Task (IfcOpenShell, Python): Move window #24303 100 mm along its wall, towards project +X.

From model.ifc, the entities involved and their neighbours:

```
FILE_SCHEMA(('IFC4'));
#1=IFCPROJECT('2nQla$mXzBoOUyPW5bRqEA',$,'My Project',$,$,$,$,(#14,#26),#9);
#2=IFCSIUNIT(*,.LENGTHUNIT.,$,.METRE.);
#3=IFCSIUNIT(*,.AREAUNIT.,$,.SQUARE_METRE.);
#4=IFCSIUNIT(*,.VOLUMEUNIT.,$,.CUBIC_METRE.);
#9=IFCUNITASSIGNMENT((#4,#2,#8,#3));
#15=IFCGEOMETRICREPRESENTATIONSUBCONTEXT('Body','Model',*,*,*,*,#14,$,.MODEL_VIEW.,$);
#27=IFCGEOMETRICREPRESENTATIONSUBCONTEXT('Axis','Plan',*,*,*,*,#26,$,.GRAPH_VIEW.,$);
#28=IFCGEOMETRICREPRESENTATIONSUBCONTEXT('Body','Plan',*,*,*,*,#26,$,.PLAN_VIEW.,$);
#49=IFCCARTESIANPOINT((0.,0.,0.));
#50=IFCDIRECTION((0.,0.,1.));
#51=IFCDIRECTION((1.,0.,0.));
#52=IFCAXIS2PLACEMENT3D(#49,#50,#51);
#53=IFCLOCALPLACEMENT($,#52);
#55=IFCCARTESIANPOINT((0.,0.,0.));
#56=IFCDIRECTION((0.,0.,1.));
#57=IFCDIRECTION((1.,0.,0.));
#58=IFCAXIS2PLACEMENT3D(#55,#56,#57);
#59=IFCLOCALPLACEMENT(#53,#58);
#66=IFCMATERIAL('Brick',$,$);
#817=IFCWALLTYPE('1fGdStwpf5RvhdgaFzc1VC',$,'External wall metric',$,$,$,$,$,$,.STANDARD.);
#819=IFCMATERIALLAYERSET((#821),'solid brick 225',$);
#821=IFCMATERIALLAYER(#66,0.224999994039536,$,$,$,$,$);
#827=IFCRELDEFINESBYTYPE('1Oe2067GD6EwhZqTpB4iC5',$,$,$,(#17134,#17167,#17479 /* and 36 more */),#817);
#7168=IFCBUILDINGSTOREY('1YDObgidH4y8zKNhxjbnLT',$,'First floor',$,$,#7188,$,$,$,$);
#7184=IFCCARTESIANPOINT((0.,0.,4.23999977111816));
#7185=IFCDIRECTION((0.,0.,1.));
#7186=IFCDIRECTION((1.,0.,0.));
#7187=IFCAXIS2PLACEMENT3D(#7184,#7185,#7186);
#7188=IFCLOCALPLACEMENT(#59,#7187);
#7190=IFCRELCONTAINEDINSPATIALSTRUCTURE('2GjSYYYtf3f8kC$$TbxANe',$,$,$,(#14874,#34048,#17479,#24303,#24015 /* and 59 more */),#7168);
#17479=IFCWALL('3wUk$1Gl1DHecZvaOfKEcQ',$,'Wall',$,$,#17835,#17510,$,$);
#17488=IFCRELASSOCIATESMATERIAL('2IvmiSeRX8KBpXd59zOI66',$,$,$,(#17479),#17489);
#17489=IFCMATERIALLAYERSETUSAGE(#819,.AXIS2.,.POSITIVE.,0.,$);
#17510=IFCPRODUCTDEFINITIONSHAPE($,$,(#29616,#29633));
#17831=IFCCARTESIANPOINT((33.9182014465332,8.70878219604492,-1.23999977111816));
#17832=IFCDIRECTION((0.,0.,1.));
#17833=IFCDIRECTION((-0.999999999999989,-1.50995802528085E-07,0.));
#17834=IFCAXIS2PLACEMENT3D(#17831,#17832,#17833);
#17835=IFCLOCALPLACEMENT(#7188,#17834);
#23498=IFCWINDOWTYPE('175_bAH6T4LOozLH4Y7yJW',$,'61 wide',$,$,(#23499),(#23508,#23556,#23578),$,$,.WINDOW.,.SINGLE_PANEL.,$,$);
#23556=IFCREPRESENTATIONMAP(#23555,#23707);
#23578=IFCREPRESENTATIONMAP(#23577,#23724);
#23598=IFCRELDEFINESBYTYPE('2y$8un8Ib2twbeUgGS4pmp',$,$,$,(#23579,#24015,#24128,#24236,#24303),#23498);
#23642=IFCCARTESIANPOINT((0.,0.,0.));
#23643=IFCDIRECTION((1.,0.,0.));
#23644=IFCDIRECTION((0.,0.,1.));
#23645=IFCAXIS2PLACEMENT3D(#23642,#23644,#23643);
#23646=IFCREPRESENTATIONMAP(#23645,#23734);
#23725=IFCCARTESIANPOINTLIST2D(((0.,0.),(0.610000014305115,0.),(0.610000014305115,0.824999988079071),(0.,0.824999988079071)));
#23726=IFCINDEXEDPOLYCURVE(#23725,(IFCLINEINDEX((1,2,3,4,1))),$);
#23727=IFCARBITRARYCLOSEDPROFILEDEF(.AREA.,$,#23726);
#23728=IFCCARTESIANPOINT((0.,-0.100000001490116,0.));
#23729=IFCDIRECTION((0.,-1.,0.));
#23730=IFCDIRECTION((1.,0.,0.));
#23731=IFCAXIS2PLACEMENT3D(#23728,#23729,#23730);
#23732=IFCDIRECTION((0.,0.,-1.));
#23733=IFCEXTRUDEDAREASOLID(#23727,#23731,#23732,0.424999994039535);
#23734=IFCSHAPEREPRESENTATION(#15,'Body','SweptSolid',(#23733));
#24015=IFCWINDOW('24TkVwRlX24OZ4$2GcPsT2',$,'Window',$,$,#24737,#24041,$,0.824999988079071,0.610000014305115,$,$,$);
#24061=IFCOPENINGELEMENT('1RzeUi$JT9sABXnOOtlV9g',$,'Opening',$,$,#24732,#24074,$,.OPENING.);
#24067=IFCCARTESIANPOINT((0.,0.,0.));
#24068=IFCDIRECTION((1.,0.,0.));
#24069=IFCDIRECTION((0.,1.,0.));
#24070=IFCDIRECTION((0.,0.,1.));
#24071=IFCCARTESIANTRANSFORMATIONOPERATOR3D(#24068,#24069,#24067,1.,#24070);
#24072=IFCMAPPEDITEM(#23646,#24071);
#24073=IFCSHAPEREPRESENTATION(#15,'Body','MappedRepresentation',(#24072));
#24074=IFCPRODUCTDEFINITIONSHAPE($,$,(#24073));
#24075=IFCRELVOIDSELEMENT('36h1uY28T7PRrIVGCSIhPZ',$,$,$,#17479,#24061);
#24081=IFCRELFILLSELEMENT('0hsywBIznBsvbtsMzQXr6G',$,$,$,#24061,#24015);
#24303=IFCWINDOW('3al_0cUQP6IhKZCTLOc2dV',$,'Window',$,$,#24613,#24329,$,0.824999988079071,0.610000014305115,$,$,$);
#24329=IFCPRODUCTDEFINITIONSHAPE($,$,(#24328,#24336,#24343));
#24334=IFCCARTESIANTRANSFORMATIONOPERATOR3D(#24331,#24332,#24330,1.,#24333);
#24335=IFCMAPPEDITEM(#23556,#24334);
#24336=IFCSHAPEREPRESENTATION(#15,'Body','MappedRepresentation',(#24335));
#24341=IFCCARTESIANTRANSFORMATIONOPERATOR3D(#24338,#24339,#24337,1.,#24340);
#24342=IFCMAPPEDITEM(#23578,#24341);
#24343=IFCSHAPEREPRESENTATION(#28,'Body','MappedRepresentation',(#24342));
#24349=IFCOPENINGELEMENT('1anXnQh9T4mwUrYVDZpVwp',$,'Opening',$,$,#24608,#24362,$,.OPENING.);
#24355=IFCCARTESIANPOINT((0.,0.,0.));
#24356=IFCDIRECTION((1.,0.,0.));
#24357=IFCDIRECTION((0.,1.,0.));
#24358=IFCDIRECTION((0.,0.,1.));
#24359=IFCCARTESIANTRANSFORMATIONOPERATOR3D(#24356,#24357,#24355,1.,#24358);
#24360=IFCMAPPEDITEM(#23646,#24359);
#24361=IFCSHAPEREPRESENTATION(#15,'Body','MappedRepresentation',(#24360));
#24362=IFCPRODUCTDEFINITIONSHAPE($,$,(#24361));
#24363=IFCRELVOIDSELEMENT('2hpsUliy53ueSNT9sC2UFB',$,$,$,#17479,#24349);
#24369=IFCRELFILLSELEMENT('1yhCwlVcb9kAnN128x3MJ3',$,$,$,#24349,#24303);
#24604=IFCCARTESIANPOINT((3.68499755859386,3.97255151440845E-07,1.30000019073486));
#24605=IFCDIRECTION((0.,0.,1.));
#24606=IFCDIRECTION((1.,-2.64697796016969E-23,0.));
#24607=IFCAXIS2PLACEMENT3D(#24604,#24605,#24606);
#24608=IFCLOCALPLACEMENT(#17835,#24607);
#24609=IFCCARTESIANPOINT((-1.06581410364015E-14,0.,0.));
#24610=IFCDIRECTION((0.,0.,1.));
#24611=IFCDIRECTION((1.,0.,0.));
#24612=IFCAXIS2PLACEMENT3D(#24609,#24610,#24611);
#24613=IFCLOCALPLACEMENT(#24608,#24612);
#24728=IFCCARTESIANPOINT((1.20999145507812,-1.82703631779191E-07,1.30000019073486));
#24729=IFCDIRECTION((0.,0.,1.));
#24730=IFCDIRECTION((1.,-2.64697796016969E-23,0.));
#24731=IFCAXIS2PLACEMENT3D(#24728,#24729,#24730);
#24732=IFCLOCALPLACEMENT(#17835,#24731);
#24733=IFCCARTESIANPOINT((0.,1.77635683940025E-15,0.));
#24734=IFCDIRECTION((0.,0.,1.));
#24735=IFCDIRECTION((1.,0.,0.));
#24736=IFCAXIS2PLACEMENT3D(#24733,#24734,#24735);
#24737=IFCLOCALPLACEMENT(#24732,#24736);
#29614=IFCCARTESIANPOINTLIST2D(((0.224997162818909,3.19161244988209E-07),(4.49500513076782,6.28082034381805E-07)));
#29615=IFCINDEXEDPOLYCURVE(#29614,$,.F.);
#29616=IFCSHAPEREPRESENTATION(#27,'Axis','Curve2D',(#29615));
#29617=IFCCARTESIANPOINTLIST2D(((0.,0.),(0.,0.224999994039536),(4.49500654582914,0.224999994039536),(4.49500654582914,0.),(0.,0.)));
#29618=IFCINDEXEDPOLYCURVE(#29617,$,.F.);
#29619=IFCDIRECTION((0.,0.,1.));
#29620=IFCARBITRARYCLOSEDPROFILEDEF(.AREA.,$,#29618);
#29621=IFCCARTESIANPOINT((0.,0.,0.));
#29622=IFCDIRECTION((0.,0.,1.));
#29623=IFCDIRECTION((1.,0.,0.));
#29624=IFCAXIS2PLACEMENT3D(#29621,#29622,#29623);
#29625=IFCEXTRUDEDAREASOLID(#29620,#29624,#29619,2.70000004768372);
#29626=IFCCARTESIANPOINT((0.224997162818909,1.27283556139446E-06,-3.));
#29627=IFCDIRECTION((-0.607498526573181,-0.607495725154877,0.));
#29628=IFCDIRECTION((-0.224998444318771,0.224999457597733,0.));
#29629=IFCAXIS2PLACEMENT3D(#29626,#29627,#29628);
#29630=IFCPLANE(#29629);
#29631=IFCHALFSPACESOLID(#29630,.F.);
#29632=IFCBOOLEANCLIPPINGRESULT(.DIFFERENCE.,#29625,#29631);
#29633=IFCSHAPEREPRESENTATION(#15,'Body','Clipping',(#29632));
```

```python
import ifcopenshell
import ifcopenshell.api.geometry
import ifcopenshell.util.placement
import ifcopenshell.util.unit

model = ifcopenshell.open("model.ifc")
unit_scale = ifcopenshell.util.unit.calculate_unit_scale(model)

window = model.by_id(24303)
opening = window.FillsVoids[0].RelatingOpeningElement
wall = opening.VoidsElements[0].RelatingBuildingElement

wall_matrix = ifcopenshell.util.placement.get_local_placement(wall.ObjectPlacement)
shift = wall_matrix[:3, 0] * -0.1 / unit_scale
before = ifcopenshell.util.placement.get_local_placement(window.ObjectPlacement)[:3, 3].copy()

# The window is placed relative to its opening, so it follows when the opening moves.
matrix = ifcopenshell.util.placement.get_local_placement(opening.ObjectPlacement)
matrix[:3, 3] += shift
ifcopenshell.api.geometry.edit_object_placement(
    model, product=opening, matrix=matrix, is_si=False, should_transform_children=True
)

after = ifcopenshell.util.placement.get_local_placement(window.ObjectPlacement)[:3, 3]
print("window moved by", (after - before).round(3) + 0.0)

model.write("model_v2.ifc")
```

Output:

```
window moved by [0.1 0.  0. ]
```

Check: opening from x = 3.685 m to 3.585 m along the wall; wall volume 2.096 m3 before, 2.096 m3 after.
